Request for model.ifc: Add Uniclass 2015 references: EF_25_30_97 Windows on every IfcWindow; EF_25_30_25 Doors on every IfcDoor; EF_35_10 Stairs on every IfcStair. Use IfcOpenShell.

First a look at what the model holds.

```python
import ifcopenshell

model = ifcopenshell.open("model.ifc")
print(model.schema)
print("classifications:", [c.Name for c in model.by_type("IfcClassification")])
for ifc_class in ("IfcDoor", "IfcRoof", "IfcStair", "IfcWall", "IfcWindow"):
    print(ifc_class, len(model.by_type(ifc_class)))
```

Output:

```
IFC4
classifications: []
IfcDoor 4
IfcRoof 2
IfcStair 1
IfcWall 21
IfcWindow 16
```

```python
import ifcopenshell
import ifcopenshell.api.classification

model = ifcopenshell.open("model.ifc")

system = ifcopenshell.api.classification.add_classification(model, classification="Uniclass 2015")

codes = {
    "IfcWindow": ("EF_25_30_97", "Windows"),
    "IfcDoor": ("EF_25_30_25", "Doors"),
    "IfcStair": ("EF_35_10", "Stairs"),
}
for ifc_class, (code, name) in codes.items():
    products = model.by_type(ifc_class)
    ifcopenshell.api.classification.add_reference(
        model, products=products, classification=system, identification=code, name=name
    )
    print(code, len(products))

model.write("model_edited.ifc")
```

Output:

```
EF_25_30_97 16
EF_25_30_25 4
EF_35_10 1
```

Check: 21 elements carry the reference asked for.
